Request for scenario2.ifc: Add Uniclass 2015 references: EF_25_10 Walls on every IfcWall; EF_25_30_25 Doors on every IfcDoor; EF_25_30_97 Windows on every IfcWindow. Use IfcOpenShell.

First a look at what the model holds.

```python
import ifcopenshell

model = ifcopenshell.open("scenario2.ifc")
print(model.schema)
print("classifications:", [c.Name for c in model.by_type("IfcClassification")])
for ifc_class in ("IfcDoor", "IfcRoof", "IfcStair", "IfcWall", "IfcWindow"):
    print(ifc_class, len(model.by_type(ifc_class)))
```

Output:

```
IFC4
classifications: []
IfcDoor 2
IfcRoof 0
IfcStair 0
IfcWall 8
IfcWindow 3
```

```python
import ifcopenshell
import ifcopenshell.api.classification

model = ifcopenshell.open("scenario2.ifc")

system = ifcopenshell.api.classification.add_classification(model, classification="Uniclass 2015")

codes = {
    "IfcWall": ("EF_25_10", "Walls"),
    "IfcDoor": ("EF_25_30_25", "Doors"),
    "IfcWindow": ("EF_25_30_97", "Windows"),
}
for ifc_class, (code, name) in codes.items():
    products = model.by_type(ifc_class)
    ifcopenshell.api.classification.add_reference(
        model, products=products, classification=system, identification=code, name=name
    )
    print(code, len(products))

model.write("scenario2_v2.ifc")
```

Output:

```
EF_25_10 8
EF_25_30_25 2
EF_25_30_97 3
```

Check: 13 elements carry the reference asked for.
